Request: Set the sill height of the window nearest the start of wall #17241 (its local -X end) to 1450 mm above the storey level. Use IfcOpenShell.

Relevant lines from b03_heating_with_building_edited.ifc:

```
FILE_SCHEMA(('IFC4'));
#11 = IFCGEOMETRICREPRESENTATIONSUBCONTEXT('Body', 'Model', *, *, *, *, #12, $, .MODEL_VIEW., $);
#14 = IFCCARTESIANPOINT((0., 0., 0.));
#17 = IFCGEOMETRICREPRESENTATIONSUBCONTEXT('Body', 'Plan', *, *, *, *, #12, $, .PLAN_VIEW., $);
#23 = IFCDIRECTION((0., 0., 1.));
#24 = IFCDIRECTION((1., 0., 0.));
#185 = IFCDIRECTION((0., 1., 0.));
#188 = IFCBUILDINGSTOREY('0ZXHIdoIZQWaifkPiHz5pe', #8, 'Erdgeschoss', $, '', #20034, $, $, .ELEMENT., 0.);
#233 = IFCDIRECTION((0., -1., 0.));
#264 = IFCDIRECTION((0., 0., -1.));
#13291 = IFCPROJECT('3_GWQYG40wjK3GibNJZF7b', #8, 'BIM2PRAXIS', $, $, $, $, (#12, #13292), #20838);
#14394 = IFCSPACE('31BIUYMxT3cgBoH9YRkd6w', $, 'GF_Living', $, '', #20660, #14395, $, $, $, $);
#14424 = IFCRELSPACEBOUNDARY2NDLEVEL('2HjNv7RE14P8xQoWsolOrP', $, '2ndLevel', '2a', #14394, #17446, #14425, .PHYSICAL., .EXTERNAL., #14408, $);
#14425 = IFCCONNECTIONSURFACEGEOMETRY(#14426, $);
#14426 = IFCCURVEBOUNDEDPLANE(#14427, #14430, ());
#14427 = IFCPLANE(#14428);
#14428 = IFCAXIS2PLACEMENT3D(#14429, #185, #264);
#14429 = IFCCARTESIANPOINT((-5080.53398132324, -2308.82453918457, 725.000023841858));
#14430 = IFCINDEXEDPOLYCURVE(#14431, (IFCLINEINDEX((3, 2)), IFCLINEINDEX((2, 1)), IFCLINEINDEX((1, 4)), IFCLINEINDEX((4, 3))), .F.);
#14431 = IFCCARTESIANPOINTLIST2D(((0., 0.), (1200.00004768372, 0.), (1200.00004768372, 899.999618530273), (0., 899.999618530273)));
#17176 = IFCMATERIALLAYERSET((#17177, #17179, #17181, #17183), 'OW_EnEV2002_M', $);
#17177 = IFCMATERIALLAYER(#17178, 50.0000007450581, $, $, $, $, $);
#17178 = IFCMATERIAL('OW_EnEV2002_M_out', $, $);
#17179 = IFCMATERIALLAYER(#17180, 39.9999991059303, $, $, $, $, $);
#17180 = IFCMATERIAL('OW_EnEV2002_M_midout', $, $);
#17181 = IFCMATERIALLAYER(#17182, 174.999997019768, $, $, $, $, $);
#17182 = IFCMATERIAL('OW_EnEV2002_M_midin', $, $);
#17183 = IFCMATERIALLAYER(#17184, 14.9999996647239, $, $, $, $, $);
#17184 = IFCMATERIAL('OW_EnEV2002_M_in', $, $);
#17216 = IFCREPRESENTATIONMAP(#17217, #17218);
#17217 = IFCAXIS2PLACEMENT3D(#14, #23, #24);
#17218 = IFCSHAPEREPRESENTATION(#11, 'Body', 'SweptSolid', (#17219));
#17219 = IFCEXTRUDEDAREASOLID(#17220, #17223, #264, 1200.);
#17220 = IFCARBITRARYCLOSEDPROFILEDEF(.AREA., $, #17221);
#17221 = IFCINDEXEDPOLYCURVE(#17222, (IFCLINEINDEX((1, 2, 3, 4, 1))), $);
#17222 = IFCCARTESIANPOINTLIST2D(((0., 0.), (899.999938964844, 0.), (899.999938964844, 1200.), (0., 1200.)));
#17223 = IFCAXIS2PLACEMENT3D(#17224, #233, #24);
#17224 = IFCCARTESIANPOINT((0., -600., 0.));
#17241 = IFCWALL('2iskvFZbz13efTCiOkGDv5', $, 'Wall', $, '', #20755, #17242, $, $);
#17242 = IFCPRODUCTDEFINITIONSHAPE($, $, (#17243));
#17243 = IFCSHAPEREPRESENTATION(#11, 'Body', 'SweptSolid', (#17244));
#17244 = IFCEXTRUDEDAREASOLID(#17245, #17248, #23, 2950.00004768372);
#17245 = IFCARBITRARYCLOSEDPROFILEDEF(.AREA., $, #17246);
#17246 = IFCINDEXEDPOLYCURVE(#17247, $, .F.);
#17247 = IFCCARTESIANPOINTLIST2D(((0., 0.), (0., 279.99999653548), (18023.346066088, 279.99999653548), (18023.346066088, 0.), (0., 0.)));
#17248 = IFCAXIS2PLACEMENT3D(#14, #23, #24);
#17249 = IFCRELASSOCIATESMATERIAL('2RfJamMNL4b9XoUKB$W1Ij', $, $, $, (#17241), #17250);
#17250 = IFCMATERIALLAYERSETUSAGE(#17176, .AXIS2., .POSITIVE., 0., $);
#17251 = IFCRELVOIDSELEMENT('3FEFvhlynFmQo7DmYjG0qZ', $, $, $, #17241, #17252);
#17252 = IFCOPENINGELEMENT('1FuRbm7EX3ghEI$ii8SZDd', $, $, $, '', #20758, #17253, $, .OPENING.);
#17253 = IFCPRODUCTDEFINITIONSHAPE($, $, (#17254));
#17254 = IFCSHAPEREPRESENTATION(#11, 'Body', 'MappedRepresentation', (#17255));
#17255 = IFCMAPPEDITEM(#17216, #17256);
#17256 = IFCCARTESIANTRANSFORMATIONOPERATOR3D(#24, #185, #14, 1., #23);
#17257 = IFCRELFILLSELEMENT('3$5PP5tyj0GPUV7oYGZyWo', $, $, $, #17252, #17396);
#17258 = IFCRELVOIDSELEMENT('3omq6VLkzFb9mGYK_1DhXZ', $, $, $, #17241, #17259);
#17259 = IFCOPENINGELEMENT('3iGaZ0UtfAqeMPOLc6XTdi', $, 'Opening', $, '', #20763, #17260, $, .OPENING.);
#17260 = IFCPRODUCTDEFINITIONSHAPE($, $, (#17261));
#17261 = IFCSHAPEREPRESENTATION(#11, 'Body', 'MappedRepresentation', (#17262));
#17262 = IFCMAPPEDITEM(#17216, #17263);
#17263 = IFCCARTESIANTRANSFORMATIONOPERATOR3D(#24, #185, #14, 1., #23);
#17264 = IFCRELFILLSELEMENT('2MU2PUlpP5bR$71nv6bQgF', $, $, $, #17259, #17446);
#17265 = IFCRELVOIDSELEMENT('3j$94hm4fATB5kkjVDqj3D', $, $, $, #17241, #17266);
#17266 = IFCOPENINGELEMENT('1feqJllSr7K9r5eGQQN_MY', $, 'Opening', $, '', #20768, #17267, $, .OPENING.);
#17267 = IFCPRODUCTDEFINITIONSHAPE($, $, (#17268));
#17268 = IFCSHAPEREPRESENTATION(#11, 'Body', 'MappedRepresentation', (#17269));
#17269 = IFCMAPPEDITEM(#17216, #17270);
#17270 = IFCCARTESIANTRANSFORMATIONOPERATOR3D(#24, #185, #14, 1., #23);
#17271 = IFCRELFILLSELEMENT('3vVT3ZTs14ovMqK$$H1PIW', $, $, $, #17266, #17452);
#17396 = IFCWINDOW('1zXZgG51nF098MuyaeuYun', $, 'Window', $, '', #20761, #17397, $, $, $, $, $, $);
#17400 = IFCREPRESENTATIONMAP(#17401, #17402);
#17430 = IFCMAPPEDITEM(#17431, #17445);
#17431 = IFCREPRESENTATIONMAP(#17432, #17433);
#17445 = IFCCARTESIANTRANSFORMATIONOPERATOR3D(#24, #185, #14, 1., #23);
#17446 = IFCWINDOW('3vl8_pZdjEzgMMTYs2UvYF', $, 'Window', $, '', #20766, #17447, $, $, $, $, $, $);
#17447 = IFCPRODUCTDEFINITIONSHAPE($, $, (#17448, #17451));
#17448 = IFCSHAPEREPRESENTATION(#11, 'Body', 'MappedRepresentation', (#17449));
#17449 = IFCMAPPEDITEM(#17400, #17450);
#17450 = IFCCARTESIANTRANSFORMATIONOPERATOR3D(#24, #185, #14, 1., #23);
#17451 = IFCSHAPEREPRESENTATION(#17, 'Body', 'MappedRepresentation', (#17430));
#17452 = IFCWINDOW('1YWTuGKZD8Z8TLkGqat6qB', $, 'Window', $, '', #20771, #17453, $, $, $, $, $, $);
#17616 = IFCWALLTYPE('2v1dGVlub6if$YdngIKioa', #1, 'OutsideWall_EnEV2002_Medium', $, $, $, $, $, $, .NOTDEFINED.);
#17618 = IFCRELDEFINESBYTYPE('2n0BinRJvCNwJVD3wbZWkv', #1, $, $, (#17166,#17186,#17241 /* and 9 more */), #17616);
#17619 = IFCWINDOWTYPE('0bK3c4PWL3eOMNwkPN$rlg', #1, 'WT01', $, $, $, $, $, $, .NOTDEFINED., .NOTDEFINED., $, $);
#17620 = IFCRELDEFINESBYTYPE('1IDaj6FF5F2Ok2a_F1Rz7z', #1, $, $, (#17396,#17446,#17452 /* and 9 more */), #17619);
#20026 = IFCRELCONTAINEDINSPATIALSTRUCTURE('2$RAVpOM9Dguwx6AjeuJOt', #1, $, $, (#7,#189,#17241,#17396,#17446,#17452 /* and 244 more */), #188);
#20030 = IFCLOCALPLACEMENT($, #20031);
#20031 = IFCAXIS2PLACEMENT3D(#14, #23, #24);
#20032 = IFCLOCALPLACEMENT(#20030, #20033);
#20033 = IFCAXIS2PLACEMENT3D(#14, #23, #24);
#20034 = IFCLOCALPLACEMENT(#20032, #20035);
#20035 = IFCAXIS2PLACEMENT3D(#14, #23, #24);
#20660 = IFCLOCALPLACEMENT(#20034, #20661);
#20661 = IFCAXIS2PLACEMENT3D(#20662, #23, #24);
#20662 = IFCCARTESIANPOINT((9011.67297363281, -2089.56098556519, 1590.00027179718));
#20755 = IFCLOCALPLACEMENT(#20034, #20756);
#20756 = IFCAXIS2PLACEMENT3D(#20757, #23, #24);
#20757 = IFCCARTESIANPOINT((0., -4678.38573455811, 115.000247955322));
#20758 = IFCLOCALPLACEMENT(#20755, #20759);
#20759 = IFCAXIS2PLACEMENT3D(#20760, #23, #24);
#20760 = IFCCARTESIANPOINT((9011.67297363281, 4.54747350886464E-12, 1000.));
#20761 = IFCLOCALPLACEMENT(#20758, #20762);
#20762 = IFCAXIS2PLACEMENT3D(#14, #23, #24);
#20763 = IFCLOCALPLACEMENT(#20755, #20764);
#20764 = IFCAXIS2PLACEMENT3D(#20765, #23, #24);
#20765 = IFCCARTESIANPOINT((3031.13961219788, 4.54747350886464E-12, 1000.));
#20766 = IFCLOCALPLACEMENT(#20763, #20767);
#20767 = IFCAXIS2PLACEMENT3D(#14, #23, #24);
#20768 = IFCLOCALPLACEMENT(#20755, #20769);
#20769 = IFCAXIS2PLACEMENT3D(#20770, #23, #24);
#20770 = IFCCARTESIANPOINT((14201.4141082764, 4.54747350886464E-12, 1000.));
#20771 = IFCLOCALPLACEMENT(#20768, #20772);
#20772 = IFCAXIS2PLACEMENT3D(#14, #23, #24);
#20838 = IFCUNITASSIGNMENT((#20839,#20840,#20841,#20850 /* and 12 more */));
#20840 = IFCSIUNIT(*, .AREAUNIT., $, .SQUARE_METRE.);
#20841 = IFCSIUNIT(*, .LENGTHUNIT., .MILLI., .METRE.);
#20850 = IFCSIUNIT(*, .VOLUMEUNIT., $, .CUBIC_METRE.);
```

```python
import numpy as np
import ifcopenshell
import ifcopenshell.api.geometry
import ifcopenshell.geom
import ifcopenshell.util.element
import ifcopenshell.util.placement
import ifcopenshell.util.shape
import ifcopenshell.util.unit

model = ifcopenshell.open("b03_heating_with_building_edited.ifc")
unit_scale = ifcopenshell.util.unit.calculate_unit_scale(model)

window = model.by_id(17446)
opening = window.FillsVoids[0].RelatingOpeningElement
storey = ifcopenshell.util.element.get_container(window, ifc_class="IfcBuildingStorey")
level = ifcopenshell.util.placement.get_local_placement(storey.ObjectPlacement)[2, 3]

# The opening's origin need not be at the sill, so measure its lowest point.
shape = ifcopenshell.geom.create_shape(ifcopenshell.geom.settings(), opening)
bottom = ifcopenshell.util.shape.get_shape_bottom_elevation(shape, shape.geometry) / unit_scale
dz = level + 1.45 / unit_scale - bottom

shift = np.array([0.0, 0.0, dz])
# The window is placed relative to its opening, so it follows when the opening moves.
matrix = ifcopenshell.util.placement.get_local_placement(opening.ObjectPlacement)
matrix[:3, 3] += shift
ifcopenshell.api.geometry.edit_object_placement(
    model, product=opening, matrix=matrix, is_si=False, should_transform_children=True
)

# Space boundary surfaces are stored in each space's coordinates; move them too.
for rel in window.ProvidesBoundaries:
    if not rel.ConnectionGeometry:
        continue
    surface = rel.ConnectionGeometry.SurfaceOnRelatingElement.BasisSurface
    space_matrix = ifcopenshell.util.placement.get_local_placement(rel.RelatingSpace.ObjectPlacement)
    point = np.array(surface.Position.Location.Coordinates) + space_matrix[:3, :3].T @ shift
    surface.Position = model.createIfcAxis2Placement3D(
        model.createIfcCartesianPoint(point.tolist()), surface.Position.Axis, surface.Position.RefDirection
    )

print(f"moved by {dz * unit_scale:+.3f} m")

model.write("b03_heating_with_building_edited_v2.ifc")
```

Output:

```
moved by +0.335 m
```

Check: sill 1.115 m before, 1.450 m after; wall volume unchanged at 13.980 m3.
